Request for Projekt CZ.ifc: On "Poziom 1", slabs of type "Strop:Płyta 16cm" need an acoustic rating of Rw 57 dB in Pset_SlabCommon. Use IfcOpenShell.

First a look at what the model holds.

```python
import ifcopenshell
import ifcopenshell.util.element

model = ifcopenshell.open("Projekt CZ.ifc")
print(model.schema)
storey = next(s for s in model.by_type("IfcBuildingStorey") if s.Name == "Poziom 1")
slabs = [e for e in ifcopenshell.util.element.get_decomposition(storey) if e.is_a("IfcSlab")]
seen = {}
for e in slabs:
    element_type = ifcopenshell.util.element.get_type(e)
    key = (element_type.Name if element_type != e and element_type else None, ifcopenshell.util.element.get_pset(e, "Pset_SlabCommon", "AcousticRating"))
    seen[key] = seen.get(key, 0) + 1
for (name, value), count in sorted(seen.items(), key=str):
    print(count, "x", name, "|", value)
```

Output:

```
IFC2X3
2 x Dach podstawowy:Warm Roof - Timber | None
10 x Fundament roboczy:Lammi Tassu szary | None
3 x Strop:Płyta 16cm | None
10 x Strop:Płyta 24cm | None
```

```python
import ifcopenshell
import ifcopenshell.api.pset
import ifcopenshell.util.element

model = ifcopenshell.open("Projekt CZ.ifc")

storey = next(s for s in model.by_type("IfcBuildingStorey") if s.Name == "Poziom 1")
slabs = [e for e in ifcopenshell.util.element.get_decomposition(storey) if e.is_a("IfcSlab")]

count = 0
for e in slabs:
    element_type = ifcopenshell.util.element.get_type(e)
    if element_type in (None, e) or element_type.Name != "Strop:Płyta 16cm":
        continue
    # add_pset returns the element's existing set when there is one.
    pset = ifcopenshell.api.pset.add_pset(model, product=e, name="Pset_SlabCommon")
    ifcopenshell.api.pset.edit_pset(model, pset=pset, properties={"AcousticRating": "Rw 57 dB"})
    count += 1

print(count, "slabs updated")

model.write("Projekt CZ_rev.ifc")
```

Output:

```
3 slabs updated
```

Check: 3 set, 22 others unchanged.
